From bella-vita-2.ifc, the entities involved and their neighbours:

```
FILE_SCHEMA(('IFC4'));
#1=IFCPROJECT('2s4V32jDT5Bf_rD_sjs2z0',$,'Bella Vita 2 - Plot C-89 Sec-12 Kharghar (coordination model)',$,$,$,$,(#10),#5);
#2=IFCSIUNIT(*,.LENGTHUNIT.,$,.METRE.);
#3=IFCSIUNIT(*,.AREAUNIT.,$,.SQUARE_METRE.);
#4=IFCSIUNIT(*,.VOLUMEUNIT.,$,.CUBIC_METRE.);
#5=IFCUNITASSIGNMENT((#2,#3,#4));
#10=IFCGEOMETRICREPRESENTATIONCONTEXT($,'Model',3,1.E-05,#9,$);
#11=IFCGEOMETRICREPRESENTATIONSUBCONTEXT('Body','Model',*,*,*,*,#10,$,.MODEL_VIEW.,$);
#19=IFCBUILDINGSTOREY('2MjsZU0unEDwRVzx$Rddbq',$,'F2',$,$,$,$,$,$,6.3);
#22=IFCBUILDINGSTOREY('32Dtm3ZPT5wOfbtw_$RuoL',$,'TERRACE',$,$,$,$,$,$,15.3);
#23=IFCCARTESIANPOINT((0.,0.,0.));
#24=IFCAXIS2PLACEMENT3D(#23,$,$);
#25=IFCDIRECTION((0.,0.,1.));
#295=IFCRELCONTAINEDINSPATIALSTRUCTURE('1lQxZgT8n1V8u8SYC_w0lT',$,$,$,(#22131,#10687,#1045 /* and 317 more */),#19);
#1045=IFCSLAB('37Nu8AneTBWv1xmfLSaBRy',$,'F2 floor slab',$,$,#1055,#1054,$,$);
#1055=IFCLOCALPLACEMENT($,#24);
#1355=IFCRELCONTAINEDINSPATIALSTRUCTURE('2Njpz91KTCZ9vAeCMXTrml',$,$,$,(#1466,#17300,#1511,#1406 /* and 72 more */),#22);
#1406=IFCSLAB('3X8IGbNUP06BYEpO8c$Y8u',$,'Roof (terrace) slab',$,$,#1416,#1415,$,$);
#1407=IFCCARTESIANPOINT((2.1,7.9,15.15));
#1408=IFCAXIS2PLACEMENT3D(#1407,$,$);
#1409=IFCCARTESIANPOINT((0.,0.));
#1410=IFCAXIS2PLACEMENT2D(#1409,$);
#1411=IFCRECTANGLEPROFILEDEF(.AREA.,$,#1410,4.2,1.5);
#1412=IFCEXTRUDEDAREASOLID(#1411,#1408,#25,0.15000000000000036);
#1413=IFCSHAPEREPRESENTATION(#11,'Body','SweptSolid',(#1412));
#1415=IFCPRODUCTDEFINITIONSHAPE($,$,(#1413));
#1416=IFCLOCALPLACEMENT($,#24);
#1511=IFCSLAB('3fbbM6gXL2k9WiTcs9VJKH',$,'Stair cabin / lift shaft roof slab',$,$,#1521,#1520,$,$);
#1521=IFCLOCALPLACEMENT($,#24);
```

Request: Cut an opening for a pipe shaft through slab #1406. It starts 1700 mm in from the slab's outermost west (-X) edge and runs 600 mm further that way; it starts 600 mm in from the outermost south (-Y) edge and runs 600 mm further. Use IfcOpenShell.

```python
import numpy as np
import ifcopenshell
import ifcopenshell.api.feature
import ifcopenshell.api.geometry
import ifcopenshell.api.root
import ifcopenshell.geom
import ifcopenshell.util.placement
import ifcopenshell.util.representation
import ifcopenshell.util.shape
import ifcopenshell.util.unit

model = ifcopenshell.open("bella-vita-2.ifc")
unit_scale = ifcopenshell.util.unit.calculate_unit_scale(model)
settings = ifcopenshell.geom.settings()


def volume(element):
    """Net volume in cubic metres, openings subtracted."""
    shape = ifcopenshell.geom.create_shape(settings, element)
    return ifcopenshell.util.shape.get_volume(shape.geometry)


slab = model.by_guid("3X8IGbNUP06BYEpO8c$Y8u")
before = volume(slab)

# Extent in the slab's own axes, in metres. The edges named are its -X and -Y sides.
slab_shape = ifcopenshell.geom.create_shape(settings, slab)
vertices = ifcopenshell.util.shape.get_vertices(slab_shape.geometry)
x_min, y_min, bottom = vertices.min(axis=0)
top = vertices[:, 2].max()

opening = ifcopenshell.api.root.create_entity(model, ifc_class="IfcOpeningElement", name="Pipe shaft opening", predefined_type="OPENING")
context = ifcopenshell.util.representation.get_context(model, "Model", "Body", "MODEL_VIEW")
width, depth = 0.6, 0.6
outline = [(0.0, 0.0), (width, 0.0), (width, depth), (0.0, depth), (0.0, 0.0)]
# Overshoot both faces by 50 mm so the cut is clean.
shape = ifcopenshell.api.geometry.add_slab_representation(
    model, context=context, depth=top - bottom + 0.1, polyline=outline
)
ifcopenshell.api.geometry.assign_representation(model, product=opening, representation=shape)

matrix = ifcopenshell.util.placement.get_local_placement(slab.ObjectPlacement)
matrix[:, 3] = matrix @ np.append(np.array([x_min + 1.7, y_min + 0.6, bottom - 0.05]) / unit_scale, 1.0)
ifcopenshell.api.geometry.edit_object_placement(model, product=opening, matrix=matrix, is_si=False)
ifcopenshell.api.feature.add_feature(model, feature=opening, element=slab)

after = volume(slab)

print(f"slab volume {before:.3f} -> {after:.3f} m3")

model.write("bella-vita-2-out.ifc")
```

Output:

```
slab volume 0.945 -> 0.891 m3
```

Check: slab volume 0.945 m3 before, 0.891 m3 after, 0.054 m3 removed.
